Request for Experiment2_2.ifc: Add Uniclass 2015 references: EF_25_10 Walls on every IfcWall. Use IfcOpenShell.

First a look at what the model holds.

```python
import ifcopenshell

model = ifcopenshell.open("Experiment2_2.ifc")
print(model.schema)
print("classifications:", [c.Name for c in model.by_type("IfcClassification")])
for ifc_class in ("IfcDoor", "IfcRoof", "IfcStair", "IfcWall", "IfcWindow"):
    print(ifc_class, len(model.by_type(ifc_class)))
```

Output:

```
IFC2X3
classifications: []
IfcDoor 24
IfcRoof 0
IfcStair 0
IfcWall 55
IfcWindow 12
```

```python
import ifcopenshell
import ifcopenshell.api.classification

model = ifcopenshell.open("Experiment2_2.ifc")

# IFC2X3 requires Source and Edition and has no link from the project to the system.
system = model.create_entity("IfcClassification", Source="NBS", Edition="2015", Name="Uniclass 2015")

codes = {
    "IfcWall": ("EF_25_10", "Walls"),
}
for ifc_class, (code, name) in codes.items():
    products = model.by_type(ifc_class)
    ifcopenshell.api.classification.add_reference(
        model, products=products, classification=system, identification=code, name=name
    )
    print(code, len(products))

model.write("Experiment2_2_v2.ifc")
```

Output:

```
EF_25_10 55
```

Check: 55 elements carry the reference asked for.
